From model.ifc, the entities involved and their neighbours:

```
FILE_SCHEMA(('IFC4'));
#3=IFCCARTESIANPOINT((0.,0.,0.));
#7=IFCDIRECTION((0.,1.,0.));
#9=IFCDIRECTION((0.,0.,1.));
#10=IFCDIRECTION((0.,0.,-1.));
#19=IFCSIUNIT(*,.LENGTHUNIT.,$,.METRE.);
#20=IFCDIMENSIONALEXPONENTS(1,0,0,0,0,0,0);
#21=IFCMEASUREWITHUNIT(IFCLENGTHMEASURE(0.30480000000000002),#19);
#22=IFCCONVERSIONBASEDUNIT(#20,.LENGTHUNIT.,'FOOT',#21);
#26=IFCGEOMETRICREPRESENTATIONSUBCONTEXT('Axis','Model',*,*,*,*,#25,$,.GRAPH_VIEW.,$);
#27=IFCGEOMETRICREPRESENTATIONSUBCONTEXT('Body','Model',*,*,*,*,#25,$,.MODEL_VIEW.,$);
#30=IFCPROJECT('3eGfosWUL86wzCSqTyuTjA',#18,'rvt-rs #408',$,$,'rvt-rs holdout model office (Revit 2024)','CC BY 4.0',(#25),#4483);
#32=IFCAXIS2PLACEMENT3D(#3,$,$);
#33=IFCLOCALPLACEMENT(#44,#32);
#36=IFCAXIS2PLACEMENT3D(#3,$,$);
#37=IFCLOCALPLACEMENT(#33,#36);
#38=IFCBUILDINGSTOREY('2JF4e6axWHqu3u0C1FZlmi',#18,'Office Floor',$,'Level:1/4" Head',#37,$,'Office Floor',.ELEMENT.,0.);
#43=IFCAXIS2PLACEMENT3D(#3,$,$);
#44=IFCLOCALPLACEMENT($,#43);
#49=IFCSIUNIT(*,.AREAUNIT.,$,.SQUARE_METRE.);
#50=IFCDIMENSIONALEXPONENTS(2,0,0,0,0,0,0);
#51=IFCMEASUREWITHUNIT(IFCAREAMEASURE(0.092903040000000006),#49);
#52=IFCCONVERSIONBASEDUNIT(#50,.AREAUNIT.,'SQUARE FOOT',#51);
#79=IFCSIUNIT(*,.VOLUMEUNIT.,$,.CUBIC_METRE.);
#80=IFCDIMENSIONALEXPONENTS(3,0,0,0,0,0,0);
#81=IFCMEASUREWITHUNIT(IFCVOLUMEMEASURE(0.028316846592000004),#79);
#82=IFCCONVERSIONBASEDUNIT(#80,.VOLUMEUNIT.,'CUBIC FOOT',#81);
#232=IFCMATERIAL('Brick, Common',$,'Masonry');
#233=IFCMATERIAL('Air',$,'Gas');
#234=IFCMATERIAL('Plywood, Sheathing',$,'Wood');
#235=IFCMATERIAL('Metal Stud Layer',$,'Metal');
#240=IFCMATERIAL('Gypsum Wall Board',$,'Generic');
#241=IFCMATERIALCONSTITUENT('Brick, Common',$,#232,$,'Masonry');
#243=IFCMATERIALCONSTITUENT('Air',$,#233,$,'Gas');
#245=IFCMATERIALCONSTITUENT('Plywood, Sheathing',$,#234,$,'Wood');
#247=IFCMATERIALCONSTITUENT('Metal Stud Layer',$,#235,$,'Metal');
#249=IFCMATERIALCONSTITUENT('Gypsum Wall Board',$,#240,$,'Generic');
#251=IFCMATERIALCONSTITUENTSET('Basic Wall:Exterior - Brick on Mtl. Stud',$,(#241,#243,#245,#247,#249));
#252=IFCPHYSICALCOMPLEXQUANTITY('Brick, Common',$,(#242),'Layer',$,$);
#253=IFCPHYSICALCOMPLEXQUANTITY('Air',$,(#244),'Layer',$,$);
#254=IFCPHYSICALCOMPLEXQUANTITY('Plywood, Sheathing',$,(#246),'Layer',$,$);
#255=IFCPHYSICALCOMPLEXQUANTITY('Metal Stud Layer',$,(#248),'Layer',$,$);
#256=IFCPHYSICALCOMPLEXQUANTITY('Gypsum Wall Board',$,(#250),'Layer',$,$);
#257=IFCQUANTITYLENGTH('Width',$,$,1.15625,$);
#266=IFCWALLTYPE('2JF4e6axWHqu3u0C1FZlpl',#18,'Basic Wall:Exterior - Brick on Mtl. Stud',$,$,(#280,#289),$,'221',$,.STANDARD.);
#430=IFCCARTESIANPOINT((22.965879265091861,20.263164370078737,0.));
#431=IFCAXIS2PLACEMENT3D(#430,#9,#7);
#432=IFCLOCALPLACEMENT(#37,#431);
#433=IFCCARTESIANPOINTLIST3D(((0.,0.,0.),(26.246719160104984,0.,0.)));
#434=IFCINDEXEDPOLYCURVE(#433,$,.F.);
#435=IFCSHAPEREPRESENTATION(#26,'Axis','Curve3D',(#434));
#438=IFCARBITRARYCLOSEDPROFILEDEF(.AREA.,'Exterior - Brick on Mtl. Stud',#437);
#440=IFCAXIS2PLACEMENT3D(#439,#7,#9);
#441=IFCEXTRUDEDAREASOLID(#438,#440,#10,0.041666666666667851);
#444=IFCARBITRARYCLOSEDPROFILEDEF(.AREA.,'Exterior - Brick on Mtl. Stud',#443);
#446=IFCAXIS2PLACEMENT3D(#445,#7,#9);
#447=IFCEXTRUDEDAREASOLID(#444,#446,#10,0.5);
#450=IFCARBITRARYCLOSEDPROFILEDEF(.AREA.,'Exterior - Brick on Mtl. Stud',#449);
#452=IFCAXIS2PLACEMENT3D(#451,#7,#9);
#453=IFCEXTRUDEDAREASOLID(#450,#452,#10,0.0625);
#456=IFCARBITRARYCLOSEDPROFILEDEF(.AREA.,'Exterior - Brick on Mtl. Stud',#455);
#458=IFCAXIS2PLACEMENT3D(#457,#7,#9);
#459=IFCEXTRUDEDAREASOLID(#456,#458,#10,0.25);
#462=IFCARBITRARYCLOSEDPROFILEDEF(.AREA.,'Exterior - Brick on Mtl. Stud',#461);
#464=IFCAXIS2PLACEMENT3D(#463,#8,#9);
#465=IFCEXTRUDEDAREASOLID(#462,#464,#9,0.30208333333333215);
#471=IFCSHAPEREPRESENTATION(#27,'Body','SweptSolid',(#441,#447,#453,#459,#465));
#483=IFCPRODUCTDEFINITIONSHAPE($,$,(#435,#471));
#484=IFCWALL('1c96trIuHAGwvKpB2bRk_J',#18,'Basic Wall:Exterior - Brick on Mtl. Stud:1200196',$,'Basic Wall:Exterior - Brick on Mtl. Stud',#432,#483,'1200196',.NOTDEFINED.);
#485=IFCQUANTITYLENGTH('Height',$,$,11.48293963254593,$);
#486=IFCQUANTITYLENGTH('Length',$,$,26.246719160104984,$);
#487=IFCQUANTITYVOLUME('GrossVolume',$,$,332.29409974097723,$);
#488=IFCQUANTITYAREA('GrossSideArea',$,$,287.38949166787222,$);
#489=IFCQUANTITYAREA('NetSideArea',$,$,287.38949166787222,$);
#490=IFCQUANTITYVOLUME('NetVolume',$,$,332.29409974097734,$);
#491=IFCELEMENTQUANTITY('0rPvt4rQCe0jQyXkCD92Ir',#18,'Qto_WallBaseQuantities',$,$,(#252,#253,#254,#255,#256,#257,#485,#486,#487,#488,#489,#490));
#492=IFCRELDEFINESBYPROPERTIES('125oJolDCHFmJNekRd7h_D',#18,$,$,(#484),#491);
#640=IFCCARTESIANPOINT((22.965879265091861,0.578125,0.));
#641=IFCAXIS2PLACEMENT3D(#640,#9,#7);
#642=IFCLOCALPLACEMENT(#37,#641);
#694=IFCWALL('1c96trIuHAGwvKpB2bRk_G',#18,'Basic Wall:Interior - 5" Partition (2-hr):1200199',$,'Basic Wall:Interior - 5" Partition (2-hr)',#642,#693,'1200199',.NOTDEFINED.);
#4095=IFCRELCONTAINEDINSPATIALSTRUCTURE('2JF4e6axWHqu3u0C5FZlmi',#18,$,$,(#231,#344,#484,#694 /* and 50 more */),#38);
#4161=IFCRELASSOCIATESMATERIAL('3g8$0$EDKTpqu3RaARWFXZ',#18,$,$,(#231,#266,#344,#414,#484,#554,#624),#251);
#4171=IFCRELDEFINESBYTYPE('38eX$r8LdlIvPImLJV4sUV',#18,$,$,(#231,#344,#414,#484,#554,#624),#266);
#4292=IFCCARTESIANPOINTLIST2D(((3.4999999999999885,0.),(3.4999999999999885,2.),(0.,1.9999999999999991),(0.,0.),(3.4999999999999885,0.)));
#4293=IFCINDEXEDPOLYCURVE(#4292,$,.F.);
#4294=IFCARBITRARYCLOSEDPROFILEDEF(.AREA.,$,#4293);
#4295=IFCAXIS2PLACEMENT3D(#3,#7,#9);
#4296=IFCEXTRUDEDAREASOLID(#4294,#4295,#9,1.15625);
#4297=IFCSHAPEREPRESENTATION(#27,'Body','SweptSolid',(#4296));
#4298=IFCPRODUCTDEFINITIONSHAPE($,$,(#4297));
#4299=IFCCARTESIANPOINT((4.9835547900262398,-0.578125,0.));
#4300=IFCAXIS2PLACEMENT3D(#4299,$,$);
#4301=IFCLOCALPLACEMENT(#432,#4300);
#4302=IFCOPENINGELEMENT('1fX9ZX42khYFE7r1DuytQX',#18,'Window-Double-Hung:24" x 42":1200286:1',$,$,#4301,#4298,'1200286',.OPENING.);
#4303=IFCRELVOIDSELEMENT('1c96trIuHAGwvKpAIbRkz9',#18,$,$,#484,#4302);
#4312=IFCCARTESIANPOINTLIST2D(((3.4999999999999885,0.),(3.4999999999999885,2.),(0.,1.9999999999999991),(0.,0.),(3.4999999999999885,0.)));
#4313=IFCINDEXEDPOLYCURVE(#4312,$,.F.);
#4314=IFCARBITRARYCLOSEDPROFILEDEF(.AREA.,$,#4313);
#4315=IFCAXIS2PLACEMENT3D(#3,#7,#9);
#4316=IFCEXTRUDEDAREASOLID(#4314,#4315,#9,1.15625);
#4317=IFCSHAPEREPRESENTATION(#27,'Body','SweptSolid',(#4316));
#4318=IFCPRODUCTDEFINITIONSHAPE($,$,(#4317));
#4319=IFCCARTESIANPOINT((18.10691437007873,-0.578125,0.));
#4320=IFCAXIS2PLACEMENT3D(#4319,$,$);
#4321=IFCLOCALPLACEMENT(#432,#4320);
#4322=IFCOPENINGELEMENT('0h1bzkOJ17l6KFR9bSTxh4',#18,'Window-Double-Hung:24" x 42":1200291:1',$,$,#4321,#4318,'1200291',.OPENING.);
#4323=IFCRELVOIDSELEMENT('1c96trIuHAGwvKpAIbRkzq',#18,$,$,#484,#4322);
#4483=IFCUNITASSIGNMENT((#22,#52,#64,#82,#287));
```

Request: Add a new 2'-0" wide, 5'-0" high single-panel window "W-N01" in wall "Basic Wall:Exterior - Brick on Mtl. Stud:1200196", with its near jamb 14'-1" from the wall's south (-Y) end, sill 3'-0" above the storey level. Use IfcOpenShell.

```python
import numpy as np
import ifcopenshell
import ifcopenshell.api.feature
import ifcopenshell.api.geometry
import ifcopenshell.api.pset
import ifcopenshell.api.root
import ifcopenshell.api.spatial
import ifcopenshell.geom
import ifcopenshell.util.element
import ifcopenshell.util.placement
import ifcopenshell.util.representation
import ifcopenshell.util.shape
import ifcopenshell.util.unit

model = ifcopenshell.open("model.ifc")
unit_scale = ifcopenshell.util.unit.calculate_unit_scale(model)
area_scale = ifcopenshell.util.unit.calculate_unit_scale(model, "AREAUNIT")
volume_scale = ifcopenshell.util.unit.calculate_unit_scale(model, "VOLUMEUNIT")
settings = ifcopenshell.geom.settings()


def volume(element):
    """Net volume in cubic metres, openings subtracted."""
    shape = ifcopenshell.geom.create_shape(settings, element)
    return ifcopenshell.util.shape.get_volume(shape.geometry)


wall = model.by_guid("1c96trIuHAGwvKpB2bRk_J")
storey = ifcopenshell.util.element.get_container(wall, ifc_class="IfcBuildingStorey")
context = ifcopenshell.util.representation.get_context(model, "Model", "Body", "MODEL_VIEW")
before = volume(wall)

width, height, from_end, sill = 0.6096, 1.524, 4.2926, 0.9144  # metres

# The wall runs along its own X axis, and the end named is its -X end.
wall_shape = ifcopenshell.geom.create_shape(settings, wall)
x, y, z = ifcopenshell.util.shape.get_vertices(wall_shape.geometry).T
start = x.min() + from_end
face, thickness = float(y.min()), float(y.max() - y.min())
wall_matrix = ifcopenshell.util.placement.get_local_placement(wall.ObjectPlacement)
level = ifcopenshell.util.placement.get_local_placement(storey.ObjectPlacement)[2, 3]


def in_wall(x, y):
    """Placement at x, y metres in the wall's axes, at sill height."""
    matrix = wall_matrix.copy()
    matrix[:, 3] = wall_matrix @ np.array([x / unit_scale, y / unit_scale, 0.0, 1.0])
    matrix[2, 3] = level + sill / unit_scale
    return matrix


# Opening: a box that overshoots both wall faces by 50 mm.
opening = ifcopenshell.api.root.create_entity(model, ifc_class="IfcOpeningElement", predefined_type="OPENING")
box = ifcopenshell.api.geometry.add_wall_representation(
    model, context=context, length=width, height=height, thickness=thickness + 0.1
)
ifcopenshell.api.geometry.assign_representation(model, product=opening, representation=box)
ifcopenshell.api.geometry.edit_object_placement(model, product=opening, matrix=in_wall(start, face - 0.05), is_si=False)
ifcopenshell.api.feature.add_feature(model, feature=opening, element=wall)

window = ifcopenshell.api.root.create_entity(model, ifc_class="IfcWindow", name="W-N01", predefined_type="WINDOW")
window.OverallWidth, window.OverallHeight = width / unit_scale, height / unit_scale
window.PartitioningType = "SINGLE_PANEL"
body = ifcopenshell.api.geometry.add_window_representation(
    model,
    context=context,
    overall_width=window.OverallWidth,
    overall_height=window.OverallHeight,
    partition_type="SINGLE_PANEL",
)
ifcopenshell.api.geometry.assign_representation(model, product=window, representation=body)
ifcopenshell.api.spatial.assign_container(model, products=[window], relating_structure=storey)
ifcopenshell.api.feature.add_filling(model, opening=opening, element=window)

# Centre the window in the wall's thickness.
ifcopenshell.api.geometry.edit_object_placement(model, product=window, matrix=in_wall(start, face), is_si=False)
window_shape = ifcopenshell.geom.create_shape(settings, window)
depth = ifcopenshell.util.shape.get_vertices(window_shape.geometry)[:, 1]
offset = face + thickness / 2 - (depth.min() + depth.max()) / 2
ifcopenshell.api.geometry.edit_object_placement(model, product=window, matrix=in_wall(start, offset), is_si=False)

after = volume(wall)

# Update the wall's stored quantities.
qto = model.by_id(ifcopenshell.util.element.get_pset(wall, "Qto_WallBaseQuantities", should_inherit=False)["id"])
ifcopenshell.api.pset.edit_qto(model, qto=qto, properties={
    "NetSideArea": after / thickness / area_scale,
    "NetVolume": after / volume_scale,
})

print(f"wall volume {before:.3f} -> {after:.3f} m3")

model.write("model-out.ifc")
```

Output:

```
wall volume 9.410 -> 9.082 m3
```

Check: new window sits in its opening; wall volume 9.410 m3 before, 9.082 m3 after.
